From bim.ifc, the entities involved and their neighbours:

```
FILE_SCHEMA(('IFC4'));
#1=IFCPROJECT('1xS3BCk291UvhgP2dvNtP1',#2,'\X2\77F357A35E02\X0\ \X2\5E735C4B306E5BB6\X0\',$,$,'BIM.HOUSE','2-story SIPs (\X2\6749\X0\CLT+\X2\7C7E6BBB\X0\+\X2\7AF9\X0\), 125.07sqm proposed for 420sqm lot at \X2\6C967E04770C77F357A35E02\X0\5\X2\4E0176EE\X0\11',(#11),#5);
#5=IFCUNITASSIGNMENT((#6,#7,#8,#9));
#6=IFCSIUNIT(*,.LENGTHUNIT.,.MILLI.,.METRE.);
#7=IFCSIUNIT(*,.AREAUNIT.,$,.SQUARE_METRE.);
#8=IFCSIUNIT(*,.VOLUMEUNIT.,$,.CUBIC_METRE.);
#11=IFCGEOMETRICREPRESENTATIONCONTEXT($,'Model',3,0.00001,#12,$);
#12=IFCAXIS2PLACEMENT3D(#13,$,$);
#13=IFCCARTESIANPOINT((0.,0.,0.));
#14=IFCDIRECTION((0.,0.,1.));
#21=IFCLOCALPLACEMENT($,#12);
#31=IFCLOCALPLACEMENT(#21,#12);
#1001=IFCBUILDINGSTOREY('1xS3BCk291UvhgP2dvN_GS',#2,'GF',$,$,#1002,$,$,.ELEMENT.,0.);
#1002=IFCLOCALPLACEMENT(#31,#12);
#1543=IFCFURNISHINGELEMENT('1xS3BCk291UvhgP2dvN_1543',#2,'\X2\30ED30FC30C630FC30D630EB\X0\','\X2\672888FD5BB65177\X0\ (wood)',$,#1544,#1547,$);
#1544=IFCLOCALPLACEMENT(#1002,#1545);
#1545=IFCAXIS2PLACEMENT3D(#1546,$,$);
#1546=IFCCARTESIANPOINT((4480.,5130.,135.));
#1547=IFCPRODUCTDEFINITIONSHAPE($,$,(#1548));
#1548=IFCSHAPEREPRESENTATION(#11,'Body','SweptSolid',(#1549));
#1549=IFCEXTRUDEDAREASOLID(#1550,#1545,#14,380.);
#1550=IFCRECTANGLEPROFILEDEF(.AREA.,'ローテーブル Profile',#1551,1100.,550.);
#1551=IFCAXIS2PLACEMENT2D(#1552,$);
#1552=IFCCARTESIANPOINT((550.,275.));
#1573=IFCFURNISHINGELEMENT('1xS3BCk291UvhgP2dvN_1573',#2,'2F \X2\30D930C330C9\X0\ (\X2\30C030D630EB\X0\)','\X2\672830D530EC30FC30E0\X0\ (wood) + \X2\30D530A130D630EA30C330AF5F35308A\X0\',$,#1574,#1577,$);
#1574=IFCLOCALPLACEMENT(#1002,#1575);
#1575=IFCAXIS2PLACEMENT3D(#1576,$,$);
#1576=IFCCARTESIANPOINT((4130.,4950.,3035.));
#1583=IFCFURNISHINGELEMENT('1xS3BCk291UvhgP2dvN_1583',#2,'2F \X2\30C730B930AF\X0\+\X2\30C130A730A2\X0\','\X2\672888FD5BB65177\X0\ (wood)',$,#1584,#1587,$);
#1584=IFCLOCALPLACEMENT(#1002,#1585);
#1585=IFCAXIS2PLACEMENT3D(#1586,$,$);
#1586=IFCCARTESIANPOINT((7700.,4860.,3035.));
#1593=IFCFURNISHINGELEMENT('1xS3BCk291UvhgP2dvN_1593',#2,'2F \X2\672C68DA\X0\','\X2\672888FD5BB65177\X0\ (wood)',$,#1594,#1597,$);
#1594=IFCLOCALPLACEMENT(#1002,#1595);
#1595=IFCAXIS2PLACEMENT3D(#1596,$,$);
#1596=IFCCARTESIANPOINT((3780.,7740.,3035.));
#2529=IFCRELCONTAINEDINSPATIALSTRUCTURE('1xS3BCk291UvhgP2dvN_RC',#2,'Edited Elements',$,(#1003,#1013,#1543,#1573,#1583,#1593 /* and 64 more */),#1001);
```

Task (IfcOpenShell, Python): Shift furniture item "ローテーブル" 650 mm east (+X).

```python
import ifcopenshell
import ifcopenshell.api.geometry
import ifcopenshell.util.placement

model = ifcopenshell.open("bim.ifc")

item = model.by_guid("1xS3BCk291UvhgP2dvN_1543")
matrix = ifcopenshell.util.placement.get_local_placement(item.ObjectPlacement)
matrix[0, 3] += 650.0
ifcopenshell.api.geometry.edit_object_placement(model, product=item, matrix=matrix, is_si=False)

print(ifcopenshell.util.placement.get_local_placement(item.ObjectPlacement).round(3) + 0.0)

model.write("bim_edited.ifc")
```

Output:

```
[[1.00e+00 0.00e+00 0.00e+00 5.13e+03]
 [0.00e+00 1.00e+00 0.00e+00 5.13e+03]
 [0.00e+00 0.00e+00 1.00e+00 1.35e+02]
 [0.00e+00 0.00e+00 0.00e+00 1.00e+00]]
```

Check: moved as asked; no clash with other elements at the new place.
